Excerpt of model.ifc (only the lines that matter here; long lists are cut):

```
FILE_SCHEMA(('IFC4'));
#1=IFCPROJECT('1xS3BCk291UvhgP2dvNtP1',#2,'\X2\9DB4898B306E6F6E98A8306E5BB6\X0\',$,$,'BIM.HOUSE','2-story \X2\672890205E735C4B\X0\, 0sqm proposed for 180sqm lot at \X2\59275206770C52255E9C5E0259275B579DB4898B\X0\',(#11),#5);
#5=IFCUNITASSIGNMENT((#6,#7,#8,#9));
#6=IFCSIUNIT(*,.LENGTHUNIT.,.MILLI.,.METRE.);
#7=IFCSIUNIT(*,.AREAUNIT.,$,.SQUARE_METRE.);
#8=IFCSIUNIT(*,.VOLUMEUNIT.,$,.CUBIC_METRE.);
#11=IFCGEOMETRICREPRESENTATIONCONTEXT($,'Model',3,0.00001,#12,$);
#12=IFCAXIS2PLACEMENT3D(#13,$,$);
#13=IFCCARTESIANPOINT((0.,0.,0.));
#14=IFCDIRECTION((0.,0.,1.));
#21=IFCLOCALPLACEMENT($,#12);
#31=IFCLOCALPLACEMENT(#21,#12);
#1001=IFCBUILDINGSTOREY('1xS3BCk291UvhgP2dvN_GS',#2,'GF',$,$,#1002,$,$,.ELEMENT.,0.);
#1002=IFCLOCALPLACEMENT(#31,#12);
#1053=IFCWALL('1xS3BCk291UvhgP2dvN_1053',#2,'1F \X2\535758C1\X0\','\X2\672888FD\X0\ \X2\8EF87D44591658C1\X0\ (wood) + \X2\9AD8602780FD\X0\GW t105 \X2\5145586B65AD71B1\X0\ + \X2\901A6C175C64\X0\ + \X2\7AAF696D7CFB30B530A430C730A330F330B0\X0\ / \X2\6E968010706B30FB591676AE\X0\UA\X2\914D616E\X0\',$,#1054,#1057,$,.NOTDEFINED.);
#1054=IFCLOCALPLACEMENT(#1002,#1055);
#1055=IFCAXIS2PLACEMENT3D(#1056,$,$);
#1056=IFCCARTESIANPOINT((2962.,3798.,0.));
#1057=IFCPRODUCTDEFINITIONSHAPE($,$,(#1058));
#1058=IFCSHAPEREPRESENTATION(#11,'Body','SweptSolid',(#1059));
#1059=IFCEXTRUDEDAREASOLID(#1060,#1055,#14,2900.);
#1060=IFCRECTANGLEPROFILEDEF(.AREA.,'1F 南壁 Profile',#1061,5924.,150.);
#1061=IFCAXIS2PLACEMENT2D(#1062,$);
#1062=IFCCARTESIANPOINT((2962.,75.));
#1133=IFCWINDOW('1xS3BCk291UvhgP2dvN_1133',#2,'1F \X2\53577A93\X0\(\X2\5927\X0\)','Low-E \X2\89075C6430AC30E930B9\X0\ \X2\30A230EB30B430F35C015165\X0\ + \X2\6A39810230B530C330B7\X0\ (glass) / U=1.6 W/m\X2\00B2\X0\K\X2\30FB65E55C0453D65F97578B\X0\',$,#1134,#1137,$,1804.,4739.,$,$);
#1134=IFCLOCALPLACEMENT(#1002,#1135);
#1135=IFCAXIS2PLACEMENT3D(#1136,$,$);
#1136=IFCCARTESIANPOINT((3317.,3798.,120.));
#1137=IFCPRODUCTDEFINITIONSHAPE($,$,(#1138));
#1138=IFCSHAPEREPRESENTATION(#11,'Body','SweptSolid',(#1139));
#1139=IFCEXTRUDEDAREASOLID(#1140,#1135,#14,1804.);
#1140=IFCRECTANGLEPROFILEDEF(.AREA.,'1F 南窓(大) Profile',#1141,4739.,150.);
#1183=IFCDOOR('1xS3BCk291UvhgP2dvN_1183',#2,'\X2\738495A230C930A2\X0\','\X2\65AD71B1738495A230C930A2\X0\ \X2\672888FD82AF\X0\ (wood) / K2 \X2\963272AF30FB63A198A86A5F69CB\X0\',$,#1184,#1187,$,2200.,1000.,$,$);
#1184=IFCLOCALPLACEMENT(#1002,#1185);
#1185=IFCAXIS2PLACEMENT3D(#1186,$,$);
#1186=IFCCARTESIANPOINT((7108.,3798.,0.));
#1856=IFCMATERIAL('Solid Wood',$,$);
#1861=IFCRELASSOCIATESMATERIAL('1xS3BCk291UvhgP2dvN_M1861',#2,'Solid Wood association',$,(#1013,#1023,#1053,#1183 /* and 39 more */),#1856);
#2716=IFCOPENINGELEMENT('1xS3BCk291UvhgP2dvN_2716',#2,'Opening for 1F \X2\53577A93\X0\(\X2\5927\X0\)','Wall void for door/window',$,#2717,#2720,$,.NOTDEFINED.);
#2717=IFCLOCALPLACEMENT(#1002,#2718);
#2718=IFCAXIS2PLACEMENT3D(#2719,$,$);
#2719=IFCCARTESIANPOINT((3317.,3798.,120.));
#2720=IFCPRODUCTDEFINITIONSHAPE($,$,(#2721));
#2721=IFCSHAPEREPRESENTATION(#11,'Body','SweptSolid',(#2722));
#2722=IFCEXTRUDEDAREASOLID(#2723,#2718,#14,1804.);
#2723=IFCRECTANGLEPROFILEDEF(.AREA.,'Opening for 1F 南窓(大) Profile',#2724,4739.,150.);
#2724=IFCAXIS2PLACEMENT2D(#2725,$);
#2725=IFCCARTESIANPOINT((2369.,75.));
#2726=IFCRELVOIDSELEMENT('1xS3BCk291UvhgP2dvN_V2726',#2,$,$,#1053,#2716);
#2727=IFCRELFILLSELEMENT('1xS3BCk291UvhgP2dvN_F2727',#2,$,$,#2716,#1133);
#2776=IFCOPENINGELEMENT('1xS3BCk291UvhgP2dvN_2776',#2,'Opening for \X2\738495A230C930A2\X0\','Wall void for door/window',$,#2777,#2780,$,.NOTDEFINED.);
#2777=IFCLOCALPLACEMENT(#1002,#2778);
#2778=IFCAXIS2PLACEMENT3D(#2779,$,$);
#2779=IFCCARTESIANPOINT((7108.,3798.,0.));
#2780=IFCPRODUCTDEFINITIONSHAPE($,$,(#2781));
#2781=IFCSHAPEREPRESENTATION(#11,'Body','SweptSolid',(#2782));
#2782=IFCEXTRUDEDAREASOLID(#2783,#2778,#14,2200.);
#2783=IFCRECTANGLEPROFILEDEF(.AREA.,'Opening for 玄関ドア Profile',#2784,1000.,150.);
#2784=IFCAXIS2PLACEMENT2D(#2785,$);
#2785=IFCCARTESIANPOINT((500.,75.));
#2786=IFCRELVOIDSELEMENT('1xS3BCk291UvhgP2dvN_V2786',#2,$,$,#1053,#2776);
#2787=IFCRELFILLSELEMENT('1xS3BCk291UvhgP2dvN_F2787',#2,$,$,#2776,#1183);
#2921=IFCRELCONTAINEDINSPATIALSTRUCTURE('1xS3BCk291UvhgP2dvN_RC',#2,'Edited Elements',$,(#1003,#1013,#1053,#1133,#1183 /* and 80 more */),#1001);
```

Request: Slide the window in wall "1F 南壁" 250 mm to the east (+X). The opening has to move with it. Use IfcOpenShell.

```python
import ifcopenshell
import ifcopenshell.api.geometry
import ifcopenshell.util.placement
import ifcopenshell.util.unit

model = ifcopenshell.open("model.ifc")
unit_scale = ifcopenshell.util.unit.calculate_unit_scale(model)

window = model.by_id(1133)
opening = window.FillsVoids[0].RelatingOpeningElement
wall = opening.VoidsElements[0].RelatingBuildingElement

wall_matrix = ifcopenshell.util.placement.get_local_placement(wall.ObjectPlacement)
shift = wall_matrix[:3, 0] * 0.25 / unit_scale
before = ifcopenshell.util.placement.get_local_placement(window.ObjectPlacement)[:3, 3].copy()

# The window is not placed relative to its opening, so move both.
for product in (opening, window):
    matrix = ifcopenshell.util.placement.get_local_placement(product.ObjectPlacement)
    matrix[:3, 3] += shift
    ifcopenshell.api.geometry.edit_object_placement(model, product=product, matrix=matrix, is_si=False)

after = ifcopenshell.util.placement.get_local_placement(window.ObjectPlacement)[:3, 3]
print("window moved by", (after - before).round(3) + 0.0)

model.write("model_edited.ifc")
```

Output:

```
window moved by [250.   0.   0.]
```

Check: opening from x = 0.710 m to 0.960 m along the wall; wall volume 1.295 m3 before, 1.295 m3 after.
